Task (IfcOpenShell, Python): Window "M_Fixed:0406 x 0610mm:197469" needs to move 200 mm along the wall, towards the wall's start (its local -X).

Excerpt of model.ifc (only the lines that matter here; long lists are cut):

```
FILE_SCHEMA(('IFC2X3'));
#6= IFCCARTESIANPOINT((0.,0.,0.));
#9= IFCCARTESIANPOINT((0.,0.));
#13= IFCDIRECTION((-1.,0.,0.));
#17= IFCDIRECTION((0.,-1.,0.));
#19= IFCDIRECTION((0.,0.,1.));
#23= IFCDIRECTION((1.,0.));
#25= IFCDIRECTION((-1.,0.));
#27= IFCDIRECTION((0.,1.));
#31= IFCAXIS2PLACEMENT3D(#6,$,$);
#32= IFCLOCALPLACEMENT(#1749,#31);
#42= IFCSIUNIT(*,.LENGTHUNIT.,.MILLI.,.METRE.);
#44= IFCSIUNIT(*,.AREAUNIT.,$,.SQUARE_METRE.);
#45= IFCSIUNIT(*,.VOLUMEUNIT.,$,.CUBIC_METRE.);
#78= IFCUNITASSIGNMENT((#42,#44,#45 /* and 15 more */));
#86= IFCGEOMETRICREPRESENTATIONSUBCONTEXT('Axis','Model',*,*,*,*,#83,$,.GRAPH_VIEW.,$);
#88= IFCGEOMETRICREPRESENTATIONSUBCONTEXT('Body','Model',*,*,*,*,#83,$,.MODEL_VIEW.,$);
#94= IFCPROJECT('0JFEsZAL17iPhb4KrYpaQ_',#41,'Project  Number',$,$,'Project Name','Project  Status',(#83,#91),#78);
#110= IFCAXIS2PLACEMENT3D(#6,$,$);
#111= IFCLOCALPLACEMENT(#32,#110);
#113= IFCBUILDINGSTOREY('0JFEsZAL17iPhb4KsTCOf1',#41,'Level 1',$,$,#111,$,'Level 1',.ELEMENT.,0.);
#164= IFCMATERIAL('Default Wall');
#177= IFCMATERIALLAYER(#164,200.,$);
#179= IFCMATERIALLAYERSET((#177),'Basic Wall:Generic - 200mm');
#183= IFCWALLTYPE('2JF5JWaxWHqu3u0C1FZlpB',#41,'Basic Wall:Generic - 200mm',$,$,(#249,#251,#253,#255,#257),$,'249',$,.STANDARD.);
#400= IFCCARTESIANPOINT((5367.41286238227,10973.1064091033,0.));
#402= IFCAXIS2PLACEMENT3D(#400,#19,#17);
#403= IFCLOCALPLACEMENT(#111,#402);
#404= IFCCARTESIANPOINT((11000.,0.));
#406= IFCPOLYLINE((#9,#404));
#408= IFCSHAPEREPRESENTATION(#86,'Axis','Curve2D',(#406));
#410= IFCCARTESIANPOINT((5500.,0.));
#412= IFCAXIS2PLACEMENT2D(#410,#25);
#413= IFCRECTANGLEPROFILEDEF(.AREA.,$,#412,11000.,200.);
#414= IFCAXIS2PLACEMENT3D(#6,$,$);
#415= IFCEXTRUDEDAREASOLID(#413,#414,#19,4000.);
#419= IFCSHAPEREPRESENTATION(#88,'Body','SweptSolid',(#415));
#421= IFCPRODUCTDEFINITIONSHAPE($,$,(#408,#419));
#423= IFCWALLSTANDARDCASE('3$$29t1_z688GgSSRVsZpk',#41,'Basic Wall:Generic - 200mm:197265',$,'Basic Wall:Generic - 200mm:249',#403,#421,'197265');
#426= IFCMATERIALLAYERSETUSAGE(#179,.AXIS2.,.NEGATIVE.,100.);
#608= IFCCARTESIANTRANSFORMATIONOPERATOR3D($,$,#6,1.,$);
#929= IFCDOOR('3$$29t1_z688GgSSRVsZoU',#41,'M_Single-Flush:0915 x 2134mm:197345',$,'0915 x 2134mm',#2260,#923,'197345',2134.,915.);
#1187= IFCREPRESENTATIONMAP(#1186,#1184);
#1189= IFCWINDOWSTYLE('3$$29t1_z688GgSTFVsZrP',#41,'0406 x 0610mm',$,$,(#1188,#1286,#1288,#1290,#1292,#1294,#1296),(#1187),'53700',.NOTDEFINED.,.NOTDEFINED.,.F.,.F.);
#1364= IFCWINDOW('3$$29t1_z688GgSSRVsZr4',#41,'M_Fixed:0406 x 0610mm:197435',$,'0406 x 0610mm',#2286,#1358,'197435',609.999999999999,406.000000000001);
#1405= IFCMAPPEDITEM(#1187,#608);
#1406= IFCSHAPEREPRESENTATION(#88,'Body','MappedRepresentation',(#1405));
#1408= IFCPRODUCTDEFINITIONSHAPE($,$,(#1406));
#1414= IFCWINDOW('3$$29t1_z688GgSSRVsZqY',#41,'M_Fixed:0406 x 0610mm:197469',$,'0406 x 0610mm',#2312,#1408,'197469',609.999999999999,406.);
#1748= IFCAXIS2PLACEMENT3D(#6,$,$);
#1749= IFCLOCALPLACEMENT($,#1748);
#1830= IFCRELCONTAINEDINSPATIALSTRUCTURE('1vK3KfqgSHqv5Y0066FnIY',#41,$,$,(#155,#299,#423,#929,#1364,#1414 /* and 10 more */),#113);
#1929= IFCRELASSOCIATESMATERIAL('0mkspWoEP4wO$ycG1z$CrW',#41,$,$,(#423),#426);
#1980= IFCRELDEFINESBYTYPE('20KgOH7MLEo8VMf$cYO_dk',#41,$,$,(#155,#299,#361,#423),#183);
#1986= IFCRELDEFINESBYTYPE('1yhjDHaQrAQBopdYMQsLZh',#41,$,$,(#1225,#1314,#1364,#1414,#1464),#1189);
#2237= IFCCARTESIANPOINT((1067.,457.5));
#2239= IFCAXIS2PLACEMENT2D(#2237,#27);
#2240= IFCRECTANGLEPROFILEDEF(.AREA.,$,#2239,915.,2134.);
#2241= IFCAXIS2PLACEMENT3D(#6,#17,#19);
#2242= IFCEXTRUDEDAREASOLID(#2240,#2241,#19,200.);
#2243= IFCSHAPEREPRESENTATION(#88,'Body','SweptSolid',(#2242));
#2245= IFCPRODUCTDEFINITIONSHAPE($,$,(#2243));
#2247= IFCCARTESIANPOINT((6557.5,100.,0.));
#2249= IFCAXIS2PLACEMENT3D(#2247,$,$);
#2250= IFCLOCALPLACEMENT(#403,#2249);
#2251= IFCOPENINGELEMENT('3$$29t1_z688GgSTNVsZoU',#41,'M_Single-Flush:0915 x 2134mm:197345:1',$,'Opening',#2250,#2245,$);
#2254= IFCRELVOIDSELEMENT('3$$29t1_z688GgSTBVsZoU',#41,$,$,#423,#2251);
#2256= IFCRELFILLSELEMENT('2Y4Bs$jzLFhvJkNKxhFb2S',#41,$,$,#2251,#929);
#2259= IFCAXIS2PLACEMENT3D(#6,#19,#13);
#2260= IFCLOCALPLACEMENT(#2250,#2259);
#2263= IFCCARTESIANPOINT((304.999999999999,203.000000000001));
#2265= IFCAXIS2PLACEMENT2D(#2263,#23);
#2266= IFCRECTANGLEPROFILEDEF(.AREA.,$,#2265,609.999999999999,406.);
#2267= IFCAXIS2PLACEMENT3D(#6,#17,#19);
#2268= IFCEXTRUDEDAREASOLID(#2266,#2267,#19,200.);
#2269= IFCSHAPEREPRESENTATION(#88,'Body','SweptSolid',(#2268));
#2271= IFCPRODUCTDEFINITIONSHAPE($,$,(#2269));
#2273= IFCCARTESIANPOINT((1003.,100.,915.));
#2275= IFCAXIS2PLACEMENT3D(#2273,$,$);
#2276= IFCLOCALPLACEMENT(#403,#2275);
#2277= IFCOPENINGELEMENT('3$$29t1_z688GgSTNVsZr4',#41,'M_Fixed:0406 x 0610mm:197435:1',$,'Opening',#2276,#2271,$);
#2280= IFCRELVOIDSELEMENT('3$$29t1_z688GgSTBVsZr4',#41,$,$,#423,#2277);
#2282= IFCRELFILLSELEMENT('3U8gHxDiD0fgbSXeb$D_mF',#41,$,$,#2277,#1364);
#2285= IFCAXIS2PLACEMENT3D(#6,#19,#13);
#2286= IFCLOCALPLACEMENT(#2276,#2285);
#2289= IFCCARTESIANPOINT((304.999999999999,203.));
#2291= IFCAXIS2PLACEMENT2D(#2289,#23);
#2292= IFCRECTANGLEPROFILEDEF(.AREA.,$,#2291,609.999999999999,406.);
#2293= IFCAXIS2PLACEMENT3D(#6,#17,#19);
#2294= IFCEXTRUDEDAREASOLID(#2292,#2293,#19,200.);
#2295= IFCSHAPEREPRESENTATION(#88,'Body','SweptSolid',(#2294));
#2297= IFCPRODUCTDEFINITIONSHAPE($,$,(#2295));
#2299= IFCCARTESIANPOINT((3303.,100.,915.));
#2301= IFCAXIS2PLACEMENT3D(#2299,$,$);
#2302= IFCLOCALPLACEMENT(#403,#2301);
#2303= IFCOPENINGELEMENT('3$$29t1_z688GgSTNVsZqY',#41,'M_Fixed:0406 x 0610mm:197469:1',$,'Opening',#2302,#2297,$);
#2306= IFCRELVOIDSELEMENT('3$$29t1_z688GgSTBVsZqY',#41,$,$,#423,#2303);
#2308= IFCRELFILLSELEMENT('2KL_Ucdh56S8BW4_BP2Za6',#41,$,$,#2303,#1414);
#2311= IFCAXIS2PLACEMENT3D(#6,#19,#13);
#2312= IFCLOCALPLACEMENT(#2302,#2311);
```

```python
import ifcopenshell
import ifcopenshell.api.geometry
import ifcopenshell.util.placement
import ifcopenshell.util.unit

model = ifcopenshell.open("model.ifc")
unit_scale = ifcopenshell.util.unit.calculate_unit_scale(model)

window = model.by_guid("3$$29t1_z688GgSSRVsZqY")
opening = window.FillsVoids[0].RelatingOpeningElement
wall = opening.VoidsElements[0].RelatingBuildingElement

wall_matrix = ifcopenshell.util.placement.get_local_placement(wall.ObjectPlacement)
shift = wall_matrix[:3, 0] * -0.2 / unit_scale
before = ifcopenshell.util.placement.get_local_placement(window.ObjectPlacement)[:3, 3].copy()

# The window is placed relative to its opening, so it follows when the opening moves.
matrix = ifcopenshell.util.placement.get_local_placement(opening.ObjectPlacement)
matrix[:3, 3] += shift
ifcopenshell.api.geometry.edit_object_placement(
    model, product=opening, matrix=matrix, is_si=False, should_transform_children=True
)

after = ifcopenshell.util.placement.get_local_placement(window.ObjectPlacement)[:3, 3]
print("window moved by", (after - before).round(3) + 0.0)

model.write("model_updated.ifc")
```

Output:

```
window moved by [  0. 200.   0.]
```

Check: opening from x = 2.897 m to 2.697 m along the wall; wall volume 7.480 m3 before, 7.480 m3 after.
